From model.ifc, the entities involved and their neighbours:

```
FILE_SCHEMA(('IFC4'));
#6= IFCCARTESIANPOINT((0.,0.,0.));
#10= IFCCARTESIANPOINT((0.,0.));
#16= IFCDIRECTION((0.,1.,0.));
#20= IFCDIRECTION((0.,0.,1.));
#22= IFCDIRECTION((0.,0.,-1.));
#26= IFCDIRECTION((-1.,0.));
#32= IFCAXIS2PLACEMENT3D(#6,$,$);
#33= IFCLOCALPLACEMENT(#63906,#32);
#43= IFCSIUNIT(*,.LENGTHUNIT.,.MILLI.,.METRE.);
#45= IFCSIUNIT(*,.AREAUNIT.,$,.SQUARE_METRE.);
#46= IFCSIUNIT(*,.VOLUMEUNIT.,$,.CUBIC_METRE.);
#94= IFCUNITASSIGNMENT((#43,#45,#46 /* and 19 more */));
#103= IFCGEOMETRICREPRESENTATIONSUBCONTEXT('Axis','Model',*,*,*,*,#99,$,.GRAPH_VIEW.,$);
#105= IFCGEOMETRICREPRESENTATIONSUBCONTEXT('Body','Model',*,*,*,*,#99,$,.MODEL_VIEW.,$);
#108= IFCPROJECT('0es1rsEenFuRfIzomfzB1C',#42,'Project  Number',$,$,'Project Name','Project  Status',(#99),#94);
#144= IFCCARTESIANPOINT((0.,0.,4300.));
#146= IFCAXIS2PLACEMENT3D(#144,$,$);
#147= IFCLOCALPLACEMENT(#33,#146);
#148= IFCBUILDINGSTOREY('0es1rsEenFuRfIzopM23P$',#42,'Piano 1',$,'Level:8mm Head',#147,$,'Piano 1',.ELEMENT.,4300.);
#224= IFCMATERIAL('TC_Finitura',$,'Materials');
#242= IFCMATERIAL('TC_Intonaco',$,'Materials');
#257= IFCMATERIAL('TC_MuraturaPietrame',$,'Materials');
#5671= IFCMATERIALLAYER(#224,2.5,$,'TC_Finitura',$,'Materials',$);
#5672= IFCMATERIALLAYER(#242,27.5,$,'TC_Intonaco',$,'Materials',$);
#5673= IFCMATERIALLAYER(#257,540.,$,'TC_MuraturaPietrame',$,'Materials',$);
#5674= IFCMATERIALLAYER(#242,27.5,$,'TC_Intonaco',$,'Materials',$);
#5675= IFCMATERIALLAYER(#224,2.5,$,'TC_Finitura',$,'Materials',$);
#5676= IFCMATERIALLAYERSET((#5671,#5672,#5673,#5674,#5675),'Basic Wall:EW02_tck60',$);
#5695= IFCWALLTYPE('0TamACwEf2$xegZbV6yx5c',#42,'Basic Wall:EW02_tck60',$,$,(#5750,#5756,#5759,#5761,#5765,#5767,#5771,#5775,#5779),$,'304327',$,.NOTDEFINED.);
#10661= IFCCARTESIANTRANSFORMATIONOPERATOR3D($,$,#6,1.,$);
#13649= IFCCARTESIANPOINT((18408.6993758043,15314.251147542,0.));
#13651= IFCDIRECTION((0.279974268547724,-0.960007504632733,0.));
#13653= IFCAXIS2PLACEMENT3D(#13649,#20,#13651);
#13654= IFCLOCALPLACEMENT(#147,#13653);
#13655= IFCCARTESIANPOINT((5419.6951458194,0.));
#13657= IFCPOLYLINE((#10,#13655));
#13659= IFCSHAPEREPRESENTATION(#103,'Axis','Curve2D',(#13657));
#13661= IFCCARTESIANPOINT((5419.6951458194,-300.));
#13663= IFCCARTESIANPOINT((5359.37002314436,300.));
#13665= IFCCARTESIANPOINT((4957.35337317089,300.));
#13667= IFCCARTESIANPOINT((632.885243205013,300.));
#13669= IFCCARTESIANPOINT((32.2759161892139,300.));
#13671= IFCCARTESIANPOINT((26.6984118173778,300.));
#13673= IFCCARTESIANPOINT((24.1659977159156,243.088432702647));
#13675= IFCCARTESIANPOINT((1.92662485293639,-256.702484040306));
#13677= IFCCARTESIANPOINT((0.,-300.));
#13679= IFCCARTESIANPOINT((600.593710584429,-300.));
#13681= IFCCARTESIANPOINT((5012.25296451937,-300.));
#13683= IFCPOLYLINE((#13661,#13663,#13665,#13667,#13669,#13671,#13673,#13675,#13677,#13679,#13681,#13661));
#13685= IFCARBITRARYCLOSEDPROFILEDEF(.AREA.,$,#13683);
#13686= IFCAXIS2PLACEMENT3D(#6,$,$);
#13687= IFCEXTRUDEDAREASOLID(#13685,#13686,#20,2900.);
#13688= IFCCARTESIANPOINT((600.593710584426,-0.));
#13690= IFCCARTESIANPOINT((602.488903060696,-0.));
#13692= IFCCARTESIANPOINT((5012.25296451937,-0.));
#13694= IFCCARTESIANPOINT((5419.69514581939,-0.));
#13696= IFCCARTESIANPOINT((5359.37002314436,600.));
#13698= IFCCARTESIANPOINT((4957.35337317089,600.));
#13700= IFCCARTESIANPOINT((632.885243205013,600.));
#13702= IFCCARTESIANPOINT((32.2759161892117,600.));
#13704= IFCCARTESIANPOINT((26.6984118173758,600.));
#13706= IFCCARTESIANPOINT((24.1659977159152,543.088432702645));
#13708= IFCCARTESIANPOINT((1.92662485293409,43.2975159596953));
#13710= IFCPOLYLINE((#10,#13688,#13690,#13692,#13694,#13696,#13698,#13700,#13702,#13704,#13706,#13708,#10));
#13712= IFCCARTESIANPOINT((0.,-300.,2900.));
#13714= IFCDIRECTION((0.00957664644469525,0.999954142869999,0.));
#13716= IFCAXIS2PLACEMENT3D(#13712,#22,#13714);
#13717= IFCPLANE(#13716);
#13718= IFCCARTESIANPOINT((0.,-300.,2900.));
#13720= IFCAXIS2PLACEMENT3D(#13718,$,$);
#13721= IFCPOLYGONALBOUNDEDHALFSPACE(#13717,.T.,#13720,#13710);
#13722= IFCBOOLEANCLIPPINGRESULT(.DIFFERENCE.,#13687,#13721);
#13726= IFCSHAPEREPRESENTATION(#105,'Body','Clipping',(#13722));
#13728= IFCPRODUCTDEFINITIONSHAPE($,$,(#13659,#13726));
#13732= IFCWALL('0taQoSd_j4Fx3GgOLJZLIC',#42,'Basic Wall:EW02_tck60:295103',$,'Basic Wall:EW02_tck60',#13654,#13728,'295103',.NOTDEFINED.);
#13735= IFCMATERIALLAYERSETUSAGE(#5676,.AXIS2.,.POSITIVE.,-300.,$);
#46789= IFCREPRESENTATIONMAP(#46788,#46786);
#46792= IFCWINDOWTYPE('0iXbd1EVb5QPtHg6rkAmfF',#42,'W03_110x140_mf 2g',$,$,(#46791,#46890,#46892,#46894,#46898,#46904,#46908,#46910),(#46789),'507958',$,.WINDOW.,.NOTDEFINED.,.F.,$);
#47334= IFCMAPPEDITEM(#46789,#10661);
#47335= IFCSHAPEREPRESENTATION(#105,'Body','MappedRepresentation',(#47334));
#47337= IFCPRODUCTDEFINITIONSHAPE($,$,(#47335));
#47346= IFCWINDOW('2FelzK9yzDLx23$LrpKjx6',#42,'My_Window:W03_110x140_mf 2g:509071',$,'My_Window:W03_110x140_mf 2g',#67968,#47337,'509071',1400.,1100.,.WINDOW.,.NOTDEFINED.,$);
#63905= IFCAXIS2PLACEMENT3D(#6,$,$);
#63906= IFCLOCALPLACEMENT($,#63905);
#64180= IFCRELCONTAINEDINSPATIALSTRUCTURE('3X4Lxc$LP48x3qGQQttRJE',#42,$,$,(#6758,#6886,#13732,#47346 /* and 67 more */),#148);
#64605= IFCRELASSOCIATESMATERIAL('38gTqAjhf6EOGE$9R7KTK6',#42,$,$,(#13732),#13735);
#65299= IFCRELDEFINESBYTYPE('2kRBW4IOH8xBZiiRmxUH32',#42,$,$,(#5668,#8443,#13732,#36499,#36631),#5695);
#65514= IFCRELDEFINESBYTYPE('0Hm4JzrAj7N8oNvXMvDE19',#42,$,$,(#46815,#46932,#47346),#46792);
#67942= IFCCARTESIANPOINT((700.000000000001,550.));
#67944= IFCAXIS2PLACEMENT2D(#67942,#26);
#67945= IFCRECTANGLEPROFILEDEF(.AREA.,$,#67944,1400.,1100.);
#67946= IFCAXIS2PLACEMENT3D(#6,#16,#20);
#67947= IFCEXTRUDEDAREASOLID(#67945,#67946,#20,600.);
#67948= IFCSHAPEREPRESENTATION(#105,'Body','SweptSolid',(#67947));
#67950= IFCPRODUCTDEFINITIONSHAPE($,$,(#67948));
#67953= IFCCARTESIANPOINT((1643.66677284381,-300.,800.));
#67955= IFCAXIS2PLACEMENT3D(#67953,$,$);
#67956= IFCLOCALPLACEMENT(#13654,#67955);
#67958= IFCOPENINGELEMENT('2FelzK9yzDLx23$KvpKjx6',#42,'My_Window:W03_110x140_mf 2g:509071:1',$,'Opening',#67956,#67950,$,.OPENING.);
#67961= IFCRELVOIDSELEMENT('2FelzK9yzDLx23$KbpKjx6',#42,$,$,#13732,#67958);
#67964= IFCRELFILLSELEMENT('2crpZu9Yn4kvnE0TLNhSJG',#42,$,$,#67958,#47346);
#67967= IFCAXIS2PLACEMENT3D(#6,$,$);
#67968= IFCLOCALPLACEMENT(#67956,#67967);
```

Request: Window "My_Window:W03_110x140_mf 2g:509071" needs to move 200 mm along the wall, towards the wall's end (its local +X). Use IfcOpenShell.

```python
import ifcopenshell
import ifcopenshell.api.geometry
import ifcopenshell.util.placement

model = ifcopenshell.open("model.ifc")

window = model.by_guid("2FelzK9yzDLx23$LrpKjx6")
opening = window.FillsVoids[0].RelatingOpeningElement
wall = opening.VoidsElements[0].RelatingBuildingElement

wall_matrix = ifcopenshell.util.placement.get_local_placement(wall.ObjectPlacement)
shift = wall_matrix[:3, 0] * 200.0
before = ifcopenshell.util.placement.get_local_placement(window.ObjectPlacement)[:3, 3].copy()

# The window is placed relative to its opening, so it follows when the opening moves.
matrix = ifcopenshell.util.placement.get_local_placement(opening.ObjectPlacement)
matrix[:3, 3] += shift
ifcopenshell.api.geometry.edit_object_placement(
    model, product=opening, matrix=matrix, is_si=False, should_transform_children=True
)

after = ifcopenshell.util.placement.get_local_placement(window.ObjectPlacement)[:3, 3]
print("window moved by", (after - before).round(3) + 0.0)

model.write("model_edited.ifc")
```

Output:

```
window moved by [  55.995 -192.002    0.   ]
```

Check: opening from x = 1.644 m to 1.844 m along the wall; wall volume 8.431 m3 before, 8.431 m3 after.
